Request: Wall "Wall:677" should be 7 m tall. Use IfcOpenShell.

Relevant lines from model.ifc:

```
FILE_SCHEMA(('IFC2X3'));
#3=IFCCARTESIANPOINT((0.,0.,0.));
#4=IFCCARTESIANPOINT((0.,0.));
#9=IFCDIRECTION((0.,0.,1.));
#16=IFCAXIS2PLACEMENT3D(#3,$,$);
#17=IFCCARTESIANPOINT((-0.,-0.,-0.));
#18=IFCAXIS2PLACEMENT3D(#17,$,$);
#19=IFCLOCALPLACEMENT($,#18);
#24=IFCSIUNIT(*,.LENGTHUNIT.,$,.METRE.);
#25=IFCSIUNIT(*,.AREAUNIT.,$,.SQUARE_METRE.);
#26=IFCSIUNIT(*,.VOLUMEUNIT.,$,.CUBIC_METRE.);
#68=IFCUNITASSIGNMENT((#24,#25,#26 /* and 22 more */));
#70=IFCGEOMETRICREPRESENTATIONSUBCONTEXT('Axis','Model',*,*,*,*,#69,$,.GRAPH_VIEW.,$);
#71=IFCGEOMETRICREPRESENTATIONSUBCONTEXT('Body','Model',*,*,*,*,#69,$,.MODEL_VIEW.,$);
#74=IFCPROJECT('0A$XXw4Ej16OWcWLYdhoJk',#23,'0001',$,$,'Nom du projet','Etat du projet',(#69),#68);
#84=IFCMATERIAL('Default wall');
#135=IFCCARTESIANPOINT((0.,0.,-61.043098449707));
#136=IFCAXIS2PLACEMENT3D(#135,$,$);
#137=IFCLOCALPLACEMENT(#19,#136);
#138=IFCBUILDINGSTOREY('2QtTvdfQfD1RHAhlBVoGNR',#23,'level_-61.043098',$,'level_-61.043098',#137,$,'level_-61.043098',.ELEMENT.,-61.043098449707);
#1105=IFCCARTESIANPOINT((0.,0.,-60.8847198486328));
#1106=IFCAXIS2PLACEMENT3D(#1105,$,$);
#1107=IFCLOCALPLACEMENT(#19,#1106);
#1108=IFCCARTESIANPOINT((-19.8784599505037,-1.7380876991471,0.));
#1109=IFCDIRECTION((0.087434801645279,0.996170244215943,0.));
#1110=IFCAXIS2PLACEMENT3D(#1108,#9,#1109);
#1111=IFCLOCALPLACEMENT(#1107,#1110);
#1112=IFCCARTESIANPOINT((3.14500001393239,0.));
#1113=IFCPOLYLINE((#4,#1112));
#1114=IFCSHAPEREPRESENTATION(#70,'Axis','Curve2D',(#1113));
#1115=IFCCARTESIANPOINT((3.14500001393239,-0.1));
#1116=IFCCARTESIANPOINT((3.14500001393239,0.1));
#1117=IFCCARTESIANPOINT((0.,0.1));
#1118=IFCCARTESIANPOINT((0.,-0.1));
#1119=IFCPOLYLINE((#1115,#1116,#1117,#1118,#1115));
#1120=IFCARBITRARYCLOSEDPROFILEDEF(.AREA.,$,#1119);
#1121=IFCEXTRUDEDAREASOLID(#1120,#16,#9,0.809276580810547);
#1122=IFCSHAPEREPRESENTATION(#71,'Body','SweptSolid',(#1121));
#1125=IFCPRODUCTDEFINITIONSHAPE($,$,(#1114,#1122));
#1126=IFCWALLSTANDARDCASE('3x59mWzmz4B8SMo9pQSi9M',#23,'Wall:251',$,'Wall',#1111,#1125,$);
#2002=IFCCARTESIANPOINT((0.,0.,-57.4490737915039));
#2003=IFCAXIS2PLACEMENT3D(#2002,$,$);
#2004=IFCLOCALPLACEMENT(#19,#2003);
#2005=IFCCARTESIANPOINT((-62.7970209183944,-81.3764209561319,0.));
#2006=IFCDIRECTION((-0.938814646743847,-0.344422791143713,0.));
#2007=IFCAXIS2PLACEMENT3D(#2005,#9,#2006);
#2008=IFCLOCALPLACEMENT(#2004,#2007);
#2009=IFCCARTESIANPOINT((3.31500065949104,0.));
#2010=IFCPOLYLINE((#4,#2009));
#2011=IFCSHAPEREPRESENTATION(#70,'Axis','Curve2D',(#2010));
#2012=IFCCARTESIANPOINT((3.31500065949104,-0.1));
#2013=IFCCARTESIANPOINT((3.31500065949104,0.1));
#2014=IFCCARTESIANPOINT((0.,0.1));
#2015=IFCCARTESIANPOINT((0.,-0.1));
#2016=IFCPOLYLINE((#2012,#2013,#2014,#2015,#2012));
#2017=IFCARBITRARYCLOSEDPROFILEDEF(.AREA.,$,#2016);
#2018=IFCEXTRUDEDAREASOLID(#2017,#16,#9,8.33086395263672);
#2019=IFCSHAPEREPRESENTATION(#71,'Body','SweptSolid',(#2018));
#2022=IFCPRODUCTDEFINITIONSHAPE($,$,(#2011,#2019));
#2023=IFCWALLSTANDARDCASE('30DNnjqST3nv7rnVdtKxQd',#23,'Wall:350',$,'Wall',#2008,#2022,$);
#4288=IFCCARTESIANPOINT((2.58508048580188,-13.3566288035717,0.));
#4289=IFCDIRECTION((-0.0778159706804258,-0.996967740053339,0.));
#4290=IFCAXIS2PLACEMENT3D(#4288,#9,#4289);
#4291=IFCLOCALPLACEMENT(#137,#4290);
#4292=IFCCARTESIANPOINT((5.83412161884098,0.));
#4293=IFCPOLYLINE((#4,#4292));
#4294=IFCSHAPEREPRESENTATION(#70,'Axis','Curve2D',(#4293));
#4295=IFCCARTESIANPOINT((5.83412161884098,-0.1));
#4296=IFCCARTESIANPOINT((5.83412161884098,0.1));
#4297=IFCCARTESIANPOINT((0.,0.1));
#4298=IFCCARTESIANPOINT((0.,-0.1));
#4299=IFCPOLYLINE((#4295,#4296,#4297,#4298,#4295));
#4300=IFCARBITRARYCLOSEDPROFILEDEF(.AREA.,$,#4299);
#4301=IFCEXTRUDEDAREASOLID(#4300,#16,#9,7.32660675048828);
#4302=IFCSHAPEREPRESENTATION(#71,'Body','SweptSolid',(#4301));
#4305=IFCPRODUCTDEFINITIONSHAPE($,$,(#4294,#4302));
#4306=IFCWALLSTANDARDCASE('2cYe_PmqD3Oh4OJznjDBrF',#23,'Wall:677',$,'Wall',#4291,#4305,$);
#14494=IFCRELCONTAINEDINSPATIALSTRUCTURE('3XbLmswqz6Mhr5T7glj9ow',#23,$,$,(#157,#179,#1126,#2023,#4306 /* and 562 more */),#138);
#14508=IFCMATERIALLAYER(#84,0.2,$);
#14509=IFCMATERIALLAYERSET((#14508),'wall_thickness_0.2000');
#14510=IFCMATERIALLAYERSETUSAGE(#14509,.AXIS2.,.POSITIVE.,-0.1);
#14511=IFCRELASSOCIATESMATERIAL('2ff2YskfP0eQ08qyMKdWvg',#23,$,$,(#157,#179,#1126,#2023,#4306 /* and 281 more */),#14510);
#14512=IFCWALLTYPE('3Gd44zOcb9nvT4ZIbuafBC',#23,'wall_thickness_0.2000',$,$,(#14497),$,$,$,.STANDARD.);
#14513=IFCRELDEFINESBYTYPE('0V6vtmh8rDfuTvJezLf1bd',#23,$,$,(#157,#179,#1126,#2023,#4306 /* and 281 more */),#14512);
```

```python
import ifcopenshell
import ifcopenshell.geom
import ifcopenshell.util.representation
import ifcopenshell.util.shape
import ifcopenshell.util.unit

model = ifcopenshell.open("model.ifc")
unit_scale = ifcopenshell.util.unit.calculate_unit_scale(model)
settings = ifcopenshell.geom.settings()


def volume(element):
    """Net volume in cubic metres, openings subtracted."""
    shape = ifcopenshell.geom.create_shape(settings, element)
    return ifcopenshell.util.shape.get_volume(shape.geometry)


wall = model.by_guid("2cYe_PmqD3Oh4OJznjDBrF")
before = volume(wall)

body = ifcopenshell.util.representation.get_representation(wall, "Model", "Body")
solid = body.Items[0]
old_height = solid.Depth
solid.Depth = 7 / unit_scale
after = volume(wall)

print(f"height {old_height:g} -> {solid.Depth:g}, volume {before:.3f} -> {after:.3f} m3")

model.write("model-out.ifc")
```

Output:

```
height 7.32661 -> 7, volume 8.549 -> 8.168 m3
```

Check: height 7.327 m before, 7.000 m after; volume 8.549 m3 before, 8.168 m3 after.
